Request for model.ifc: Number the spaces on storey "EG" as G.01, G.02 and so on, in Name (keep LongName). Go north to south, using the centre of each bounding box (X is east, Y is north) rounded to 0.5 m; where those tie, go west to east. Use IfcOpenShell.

First a look at what the model holds.

```python
import ifcopenshell
import ifcopenshell.util.element
import ifcopenshell.util.placement

model = ifcopenshell.open("model.ifc")
print(model.schema)
storey = next(s for s in model.by_type("IfcBuildingStorey") if s.Name == "EG")
spaces = [e for e in ifcopenshell.util.element.get_decomposition(storey) if e.is_a("IfcSpace")]
for e in sorted(spaces, key=lambda e: e.id()):
    origin = ifcopenshell.util.placement.get_local_placement(e.ObjectPlacement)[:3, 3]
    print(e.id(), e.Name, e.LongName, origin.round(2) + 0.0, sep=" | ")
```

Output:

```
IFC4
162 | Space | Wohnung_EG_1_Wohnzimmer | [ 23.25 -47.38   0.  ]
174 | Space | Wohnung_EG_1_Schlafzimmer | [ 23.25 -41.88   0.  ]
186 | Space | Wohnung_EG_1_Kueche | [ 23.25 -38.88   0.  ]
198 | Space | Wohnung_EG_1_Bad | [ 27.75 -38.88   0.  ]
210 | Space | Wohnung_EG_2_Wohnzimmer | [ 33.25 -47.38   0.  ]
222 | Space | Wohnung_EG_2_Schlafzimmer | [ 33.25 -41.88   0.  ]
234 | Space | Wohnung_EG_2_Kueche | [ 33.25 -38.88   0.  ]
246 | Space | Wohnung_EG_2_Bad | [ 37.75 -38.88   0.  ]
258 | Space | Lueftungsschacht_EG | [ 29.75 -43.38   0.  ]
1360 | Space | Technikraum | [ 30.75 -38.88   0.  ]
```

```python
import ifcopenshell
import ifcopenshell.geom
import ifcopenshell.util.element
import ifcopenshell.util.shape

model = ifcopenshell.open("model.ifc")
settings = ifcopenshell.geom.settings()
settings.set("use-world-coords", True)


def centre(element):
    shape = ifcopenshell.geom.create_shape(settings, element)
    return ifcopenshell.util.shape.get_bbox_centroid(shape.geometry)


storey = next(s for s in model.by_type("IfcBuildingStorey") if s.Name == "EG")
spaces = [e for e in ifcopenshell.util.element.get_decomposition(storey) if e.is_a("IfcSpace")]

# Insertion points can sit at a corner or the storey origin, so sort by the geometry (in metres).
centres = {e: centre(e) for e in spaces}
spaces.sort(key=lambda e: (-round(centres[e][1] / 0.5), centres[e][0]))

for i, e in enumerate(spaces, start=1):
    number = f"G.{i:02d}"
    e.Name = number
    print(e.id(), number)

model.write("model_updated.ifc")
```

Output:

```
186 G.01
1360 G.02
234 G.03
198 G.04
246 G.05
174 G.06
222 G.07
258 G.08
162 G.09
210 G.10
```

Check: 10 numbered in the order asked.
